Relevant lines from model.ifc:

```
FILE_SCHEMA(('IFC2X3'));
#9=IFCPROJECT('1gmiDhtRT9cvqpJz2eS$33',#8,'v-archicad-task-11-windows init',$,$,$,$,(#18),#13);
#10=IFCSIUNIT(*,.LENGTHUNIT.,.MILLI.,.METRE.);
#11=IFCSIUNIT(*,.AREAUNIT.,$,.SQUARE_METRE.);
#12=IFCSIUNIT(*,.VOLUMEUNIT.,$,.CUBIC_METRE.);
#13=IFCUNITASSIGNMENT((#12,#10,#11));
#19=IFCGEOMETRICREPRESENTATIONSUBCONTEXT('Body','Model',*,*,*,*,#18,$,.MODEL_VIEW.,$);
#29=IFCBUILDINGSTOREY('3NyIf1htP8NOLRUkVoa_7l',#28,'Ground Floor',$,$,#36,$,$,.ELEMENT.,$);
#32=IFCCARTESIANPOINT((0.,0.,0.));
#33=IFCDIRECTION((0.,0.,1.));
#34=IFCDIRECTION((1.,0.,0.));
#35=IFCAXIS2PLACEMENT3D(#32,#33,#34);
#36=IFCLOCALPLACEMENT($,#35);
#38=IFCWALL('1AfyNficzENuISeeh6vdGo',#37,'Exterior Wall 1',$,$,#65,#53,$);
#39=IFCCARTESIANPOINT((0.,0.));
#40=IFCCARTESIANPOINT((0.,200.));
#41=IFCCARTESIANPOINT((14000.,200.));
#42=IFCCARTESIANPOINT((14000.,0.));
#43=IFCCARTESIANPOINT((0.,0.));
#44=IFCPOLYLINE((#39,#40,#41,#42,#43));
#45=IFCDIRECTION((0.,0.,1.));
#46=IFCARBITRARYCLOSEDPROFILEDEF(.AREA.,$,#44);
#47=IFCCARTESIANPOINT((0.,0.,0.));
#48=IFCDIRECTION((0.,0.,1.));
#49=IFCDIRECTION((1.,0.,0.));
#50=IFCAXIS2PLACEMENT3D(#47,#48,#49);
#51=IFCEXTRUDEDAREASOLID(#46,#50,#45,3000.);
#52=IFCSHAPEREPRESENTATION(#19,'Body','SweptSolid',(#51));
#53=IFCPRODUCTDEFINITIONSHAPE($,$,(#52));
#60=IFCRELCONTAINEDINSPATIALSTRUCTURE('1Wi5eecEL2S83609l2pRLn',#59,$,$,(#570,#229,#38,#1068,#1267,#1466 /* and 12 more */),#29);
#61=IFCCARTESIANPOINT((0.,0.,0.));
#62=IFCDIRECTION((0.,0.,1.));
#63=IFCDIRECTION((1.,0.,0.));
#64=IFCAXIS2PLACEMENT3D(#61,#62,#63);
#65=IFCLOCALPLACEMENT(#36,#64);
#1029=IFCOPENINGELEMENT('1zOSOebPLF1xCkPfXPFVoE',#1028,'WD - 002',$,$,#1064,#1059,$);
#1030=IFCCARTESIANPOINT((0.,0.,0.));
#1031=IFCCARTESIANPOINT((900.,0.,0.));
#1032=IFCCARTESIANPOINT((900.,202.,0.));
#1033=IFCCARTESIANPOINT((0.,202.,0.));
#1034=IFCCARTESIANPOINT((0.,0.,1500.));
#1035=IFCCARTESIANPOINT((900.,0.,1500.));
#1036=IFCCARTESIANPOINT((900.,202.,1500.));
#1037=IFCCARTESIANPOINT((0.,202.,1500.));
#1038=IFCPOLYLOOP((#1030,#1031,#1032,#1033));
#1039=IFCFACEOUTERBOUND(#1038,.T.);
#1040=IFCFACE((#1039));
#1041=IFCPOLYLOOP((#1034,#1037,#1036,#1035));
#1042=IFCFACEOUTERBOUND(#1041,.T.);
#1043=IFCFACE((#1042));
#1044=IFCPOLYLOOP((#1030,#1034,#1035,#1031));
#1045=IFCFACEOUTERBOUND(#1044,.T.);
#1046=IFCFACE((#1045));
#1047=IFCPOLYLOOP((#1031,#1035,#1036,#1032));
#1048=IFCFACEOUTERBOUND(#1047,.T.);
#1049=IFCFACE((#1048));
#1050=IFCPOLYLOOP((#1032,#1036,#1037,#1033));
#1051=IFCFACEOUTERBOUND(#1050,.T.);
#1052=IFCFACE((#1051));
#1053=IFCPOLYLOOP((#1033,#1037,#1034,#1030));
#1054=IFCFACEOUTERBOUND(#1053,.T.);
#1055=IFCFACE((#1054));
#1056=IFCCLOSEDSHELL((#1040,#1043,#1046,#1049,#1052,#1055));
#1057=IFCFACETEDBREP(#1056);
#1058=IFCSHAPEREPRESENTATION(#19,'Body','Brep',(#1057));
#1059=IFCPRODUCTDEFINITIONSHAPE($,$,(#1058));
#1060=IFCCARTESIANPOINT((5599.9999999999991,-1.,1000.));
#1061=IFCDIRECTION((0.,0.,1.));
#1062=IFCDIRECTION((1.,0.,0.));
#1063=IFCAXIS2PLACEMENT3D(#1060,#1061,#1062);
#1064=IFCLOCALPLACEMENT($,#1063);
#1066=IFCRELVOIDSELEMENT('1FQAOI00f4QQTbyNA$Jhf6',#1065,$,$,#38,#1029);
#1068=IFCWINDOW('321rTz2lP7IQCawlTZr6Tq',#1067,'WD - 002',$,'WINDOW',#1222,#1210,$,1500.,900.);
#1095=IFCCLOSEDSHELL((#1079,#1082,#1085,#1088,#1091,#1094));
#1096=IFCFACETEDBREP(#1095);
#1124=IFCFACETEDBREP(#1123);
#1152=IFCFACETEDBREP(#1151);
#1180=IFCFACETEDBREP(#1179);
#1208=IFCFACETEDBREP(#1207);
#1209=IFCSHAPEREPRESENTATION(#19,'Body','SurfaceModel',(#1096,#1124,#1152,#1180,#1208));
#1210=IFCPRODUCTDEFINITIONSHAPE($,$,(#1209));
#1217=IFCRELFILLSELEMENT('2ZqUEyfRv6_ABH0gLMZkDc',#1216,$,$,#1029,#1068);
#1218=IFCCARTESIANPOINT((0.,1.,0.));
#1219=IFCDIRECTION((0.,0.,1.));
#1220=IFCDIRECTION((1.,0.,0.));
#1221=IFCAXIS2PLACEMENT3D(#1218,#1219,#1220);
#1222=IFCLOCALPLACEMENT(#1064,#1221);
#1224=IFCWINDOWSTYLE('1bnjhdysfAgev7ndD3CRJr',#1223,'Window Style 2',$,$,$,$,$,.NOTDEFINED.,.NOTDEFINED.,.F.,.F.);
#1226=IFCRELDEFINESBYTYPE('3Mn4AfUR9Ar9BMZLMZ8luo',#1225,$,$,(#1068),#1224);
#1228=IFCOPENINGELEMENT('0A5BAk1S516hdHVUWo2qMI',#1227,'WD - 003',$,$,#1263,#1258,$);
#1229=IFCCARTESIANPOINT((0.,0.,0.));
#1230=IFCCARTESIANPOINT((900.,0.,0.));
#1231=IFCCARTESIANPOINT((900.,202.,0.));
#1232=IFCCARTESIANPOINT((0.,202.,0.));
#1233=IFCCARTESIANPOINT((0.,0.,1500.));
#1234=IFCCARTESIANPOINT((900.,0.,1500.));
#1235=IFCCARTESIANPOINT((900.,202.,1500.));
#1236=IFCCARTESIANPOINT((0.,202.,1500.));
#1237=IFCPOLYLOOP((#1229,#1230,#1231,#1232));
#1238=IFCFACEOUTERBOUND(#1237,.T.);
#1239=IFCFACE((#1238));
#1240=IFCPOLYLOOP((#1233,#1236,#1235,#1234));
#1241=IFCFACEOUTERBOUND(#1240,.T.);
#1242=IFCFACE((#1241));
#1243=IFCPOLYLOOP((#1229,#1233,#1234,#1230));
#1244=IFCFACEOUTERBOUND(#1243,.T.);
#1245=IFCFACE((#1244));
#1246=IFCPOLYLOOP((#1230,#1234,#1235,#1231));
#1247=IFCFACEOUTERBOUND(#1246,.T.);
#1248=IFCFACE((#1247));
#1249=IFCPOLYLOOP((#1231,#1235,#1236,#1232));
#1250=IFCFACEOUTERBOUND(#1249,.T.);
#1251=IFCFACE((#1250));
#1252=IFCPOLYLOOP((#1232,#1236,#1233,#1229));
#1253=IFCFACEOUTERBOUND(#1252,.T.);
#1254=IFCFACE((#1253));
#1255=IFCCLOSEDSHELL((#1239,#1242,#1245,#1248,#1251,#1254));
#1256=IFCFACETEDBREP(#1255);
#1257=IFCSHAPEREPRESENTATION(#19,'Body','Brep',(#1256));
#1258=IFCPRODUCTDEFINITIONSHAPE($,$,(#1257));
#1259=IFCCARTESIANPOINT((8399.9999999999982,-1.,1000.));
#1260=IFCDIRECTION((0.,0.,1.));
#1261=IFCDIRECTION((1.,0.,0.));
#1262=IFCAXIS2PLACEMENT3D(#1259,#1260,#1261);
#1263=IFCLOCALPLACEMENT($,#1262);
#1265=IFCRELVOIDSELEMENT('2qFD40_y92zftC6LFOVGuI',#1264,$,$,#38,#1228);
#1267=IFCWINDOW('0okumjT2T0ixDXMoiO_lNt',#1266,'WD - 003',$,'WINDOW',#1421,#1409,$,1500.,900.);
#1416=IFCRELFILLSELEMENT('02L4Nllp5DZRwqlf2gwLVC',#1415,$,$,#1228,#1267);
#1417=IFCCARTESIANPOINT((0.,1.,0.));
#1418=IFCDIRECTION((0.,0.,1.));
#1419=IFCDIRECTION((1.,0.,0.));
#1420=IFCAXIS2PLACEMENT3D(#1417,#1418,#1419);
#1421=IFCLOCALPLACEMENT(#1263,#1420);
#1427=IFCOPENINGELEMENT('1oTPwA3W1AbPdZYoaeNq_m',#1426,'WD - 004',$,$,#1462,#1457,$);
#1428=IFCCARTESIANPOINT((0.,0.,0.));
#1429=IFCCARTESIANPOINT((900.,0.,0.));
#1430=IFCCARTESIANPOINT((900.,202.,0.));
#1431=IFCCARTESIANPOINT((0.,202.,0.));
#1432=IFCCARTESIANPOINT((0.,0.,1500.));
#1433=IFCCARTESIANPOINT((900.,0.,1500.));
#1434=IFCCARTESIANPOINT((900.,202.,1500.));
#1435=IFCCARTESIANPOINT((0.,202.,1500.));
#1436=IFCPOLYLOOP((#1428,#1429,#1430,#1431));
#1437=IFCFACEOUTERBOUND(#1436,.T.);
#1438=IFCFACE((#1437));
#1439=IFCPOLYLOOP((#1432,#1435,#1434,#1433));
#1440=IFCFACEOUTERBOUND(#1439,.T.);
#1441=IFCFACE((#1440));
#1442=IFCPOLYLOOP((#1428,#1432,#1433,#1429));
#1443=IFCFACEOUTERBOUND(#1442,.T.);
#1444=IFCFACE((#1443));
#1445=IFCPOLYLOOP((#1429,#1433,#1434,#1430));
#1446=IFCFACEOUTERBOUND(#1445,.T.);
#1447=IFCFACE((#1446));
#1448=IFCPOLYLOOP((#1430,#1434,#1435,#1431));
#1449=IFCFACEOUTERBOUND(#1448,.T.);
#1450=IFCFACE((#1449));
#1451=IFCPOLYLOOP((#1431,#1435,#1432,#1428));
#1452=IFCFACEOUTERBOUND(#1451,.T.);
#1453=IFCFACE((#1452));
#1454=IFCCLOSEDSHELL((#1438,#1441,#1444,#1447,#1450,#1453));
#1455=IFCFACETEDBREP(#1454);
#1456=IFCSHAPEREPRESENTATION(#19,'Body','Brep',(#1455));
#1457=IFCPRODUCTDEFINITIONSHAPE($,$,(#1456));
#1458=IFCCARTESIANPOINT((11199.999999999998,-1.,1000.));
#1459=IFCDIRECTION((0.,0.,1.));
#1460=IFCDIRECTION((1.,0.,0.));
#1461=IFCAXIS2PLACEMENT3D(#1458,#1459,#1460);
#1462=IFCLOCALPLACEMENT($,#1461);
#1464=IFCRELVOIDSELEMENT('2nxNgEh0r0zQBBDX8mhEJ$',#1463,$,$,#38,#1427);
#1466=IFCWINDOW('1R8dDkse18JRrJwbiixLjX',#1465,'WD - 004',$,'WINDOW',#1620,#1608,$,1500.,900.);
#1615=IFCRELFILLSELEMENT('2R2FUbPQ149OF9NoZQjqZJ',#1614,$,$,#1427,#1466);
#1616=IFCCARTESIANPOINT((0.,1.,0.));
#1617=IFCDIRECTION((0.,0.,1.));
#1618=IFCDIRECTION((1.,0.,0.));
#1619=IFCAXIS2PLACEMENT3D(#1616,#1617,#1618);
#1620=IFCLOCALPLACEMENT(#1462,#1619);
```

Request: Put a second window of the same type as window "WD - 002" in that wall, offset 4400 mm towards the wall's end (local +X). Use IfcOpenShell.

```python
import ifcopenshell
import ifcopenshell.api.feature
import ifcopenshell.api.geometry
import ifcopenshell.api.root
import ifcopenshell.geom
import ifcopenshell.util.element
import ifcopenshell.util.placement
import ifcopenshell.util.shape
import ifcopenshell.util.unit

model = ifcopenshell.open("model.ifc")
unit_scale = ifcopenshell.util.unit.calculate_unit_scale(model)
settings = ifcopenshell.geom.settings()


def volume(element):
    """Net volume in cubic metres, openings subtracted."""
    shape = ifcopenshell.geom.create_shape(settings, element)
    return ifcopenshell.util.shape.get_volume(shape.geometry)


window = model.by_guid("321rTz2lP7IQCawlTZr6Tq")
opening = window.FillsVoids[0].RelatingOpeningElement
wall = opening.VoidsElements[0].RelatingBuildingElement
before = volume(wall)
shift = ifcopenshell.util.placement.get_local_placement(wall.ObjectPlacement)[:3, 0] * 4.4 / unit_scale

# copy_class copies the void relationship, type, container and properties, but no geometry.
new_opening = ifcopenshell.api.root.copy_class(model, product=opening)
new_opening.Representation = ifcopenshell.util.element.copy_deep(
    model, opening.Representation, exclude=["IfcGeometricRepresentationContext", "IfcRepresentationMap"]
)
new_window = ifcopenshell.api.root.copy_class(model, product=window)
new_window.Representation = ifcopenshell.util.element.copy_deep(
    model, window.Representation, exclude=["IfcGeometricRepresentationContext", "IfcRepresentationMap"]
)
fills = ifcopenshell.api.feature.add_filling(model, opening=new_opening, element=new_window)
fills.OwnerHistory = new_window.OwnerHistory  # required in IFC2X3

for old, new in ((opening, new_opening), (window, new_window)):
    matrix = ifcopenshell.util.placement.get_local_placement(old.ObjectPlacement)
    matrix[:3, 3] += shift
    ifcopenshell.api.geometry.edit_object_placement(model, product=new, matrix=matrix, is_si=False)

after = volume(wall)

print(f"wall volume {before:.3f} -> {after:.3f} m3")

model.write("model_rev.ifc")
```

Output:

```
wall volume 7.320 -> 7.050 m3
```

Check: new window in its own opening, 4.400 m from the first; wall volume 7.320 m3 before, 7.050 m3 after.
